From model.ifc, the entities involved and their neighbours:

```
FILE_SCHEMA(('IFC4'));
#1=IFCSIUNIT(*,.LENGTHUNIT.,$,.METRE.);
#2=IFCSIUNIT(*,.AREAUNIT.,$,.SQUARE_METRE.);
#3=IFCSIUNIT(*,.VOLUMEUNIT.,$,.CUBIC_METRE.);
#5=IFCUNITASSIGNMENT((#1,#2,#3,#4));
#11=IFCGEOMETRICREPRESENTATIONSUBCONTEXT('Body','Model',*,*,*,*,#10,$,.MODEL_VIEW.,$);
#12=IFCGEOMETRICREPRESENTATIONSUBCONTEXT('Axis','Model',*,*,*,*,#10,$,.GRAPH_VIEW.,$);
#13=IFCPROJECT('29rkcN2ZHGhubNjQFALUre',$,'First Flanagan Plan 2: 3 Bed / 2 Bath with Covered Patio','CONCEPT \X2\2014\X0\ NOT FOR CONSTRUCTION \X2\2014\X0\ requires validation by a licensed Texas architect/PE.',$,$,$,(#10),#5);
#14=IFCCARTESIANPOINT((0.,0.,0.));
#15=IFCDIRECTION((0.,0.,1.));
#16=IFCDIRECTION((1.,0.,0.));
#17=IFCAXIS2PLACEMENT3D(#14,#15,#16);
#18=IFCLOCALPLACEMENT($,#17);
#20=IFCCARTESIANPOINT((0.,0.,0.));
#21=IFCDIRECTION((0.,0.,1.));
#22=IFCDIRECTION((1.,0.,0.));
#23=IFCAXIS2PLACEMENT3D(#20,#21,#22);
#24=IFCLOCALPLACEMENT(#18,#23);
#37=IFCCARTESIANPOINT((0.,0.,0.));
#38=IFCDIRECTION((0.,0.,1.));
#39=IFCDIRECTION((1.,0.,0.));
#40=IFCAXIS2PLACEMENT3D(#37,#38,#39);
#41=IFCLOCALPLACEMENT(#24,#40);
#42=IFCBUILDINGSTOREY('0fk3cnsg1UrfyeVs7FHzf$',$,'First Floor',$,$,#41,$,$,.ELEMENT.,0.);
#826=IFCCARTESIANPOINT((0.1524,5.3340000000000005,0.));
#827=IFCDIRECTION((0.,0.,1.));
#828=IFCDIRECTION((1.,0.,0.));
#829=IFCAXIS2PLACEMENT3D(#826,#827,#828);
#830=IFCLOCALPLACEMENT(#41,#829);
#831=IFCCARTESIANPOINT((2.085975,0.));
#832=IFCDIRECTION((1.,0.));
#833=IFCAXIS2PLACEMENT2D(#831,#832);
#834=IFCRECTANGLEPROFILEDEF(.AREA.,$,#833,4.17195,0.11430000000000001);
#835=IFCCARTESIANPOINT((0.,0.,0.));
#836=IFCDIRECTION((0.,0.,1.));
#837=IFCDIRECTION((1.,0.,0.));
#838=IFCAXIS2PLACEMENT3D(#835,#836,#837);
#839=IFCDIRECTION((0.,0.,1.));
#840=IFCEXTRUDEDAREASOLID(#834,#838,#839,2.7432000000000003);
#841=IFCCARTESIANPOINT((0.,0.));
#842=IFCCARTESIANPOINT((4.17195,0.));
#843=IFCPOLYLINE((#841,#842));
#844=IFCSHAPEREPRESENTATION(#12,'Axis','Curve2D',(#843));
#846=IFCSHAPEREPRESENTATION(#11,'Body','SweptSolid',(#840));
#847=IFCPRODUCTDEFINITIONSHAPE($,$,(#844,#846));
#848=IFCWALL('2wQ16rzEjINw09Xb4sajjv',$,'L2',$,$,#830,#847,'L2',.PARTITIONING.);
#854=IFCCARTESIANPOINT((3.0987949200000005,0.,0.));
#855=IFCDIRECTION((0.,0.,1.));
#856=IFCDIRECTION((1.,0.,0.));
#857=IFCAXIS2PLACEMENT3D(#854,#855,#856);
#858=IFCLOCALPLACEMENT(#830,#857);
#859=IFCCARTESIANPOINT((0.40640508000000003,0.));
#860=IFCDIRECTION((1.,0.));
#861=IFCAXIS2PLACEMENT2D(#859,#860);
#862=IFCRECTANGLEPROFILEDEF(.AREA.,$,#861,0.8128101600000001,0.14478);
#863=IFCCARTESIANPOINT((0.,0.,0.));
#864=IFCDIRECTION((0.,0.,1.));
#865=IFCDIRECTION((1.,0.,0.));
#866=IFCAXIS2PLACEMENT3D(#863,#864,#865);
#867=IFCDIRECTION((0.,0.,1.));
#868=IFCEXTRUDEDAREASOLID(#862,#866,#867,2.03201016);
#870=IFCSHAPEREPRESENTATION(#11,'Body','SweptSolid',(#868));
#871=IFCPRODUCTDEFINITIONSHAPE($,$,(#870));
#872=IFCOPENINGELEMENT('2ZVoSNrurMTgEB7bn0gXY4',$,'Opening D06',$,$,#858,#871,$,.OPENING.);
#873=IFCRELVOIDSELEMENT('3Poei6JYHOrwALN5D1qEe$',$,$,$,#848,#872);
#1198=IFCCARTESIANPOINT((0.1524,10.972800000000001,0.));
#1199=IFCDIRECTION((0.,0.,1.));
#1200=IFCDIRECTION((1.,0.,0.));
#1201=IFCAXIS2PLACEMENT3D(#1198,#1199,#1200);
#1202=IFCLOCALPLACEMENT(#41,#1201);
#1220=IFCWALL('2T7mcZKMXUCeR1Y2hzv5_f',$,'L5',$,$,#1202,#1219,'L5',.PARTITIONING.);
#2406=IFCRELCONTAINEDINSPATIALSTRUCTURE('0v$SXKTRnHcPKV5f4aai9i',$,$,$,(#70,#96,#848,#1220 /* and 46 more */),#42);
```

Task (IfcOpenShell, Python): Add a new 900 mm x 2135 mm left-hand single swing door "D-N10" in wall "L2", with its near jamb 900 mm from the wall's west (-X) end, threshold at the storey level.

```python
import numpy as np
import ifcopenshell
import ifcopenshell.api.feature
import ifcopenshell.api.geometry
import ifcopenshell.api.root
import ifcopenshell.api.spatial
import ifcopenshell.geom
import ifcopenshell.util.element
import ifcopenshell.util.placement
import ifcopenshell.util.representation
import ifcopenshell.util.shape
import ifcopenshell.util.unit

model = ifcopenshell.open("model.ifc")
unit_scale = ifcopenshell.util.unit.calculate_unit_scale(model)
settings = ifcopenshell.geom.settings()


def volume(element):
    """Net volume in cubic metres, openings subtracted."""
    shape = ifcopenshell.geom.create_shape(settings, element)
    return ifcopenshell.util.shape.get_volume(shape.geometry)


wall = model.by_id(848)
storey = ifcopenshell.util.element.get_container(wall, ifc_class="IfcBuildingStorey")
context = ifcopenshell.util.representation.get_context(model, "Model", "Body", "MODEL_VIEW")
before = volume(wall)

width, height, from_end, sill = 0.9, 2.135, 0.9, 0.0  # metres

# The wall runs along its own X axis, and the end named is its -X end.
wall_shape = ifcopenshell.geom.create_shape(settings, wall)
x, y, z = ifcopenshell.util.shape.get_vertices(wall_shape.geometry).T
start = x.min() + from_end
face, thickness = float(y.min()), float(y.max() - y.min())
wall_matrix = ifcopenshell.util.placement.get_local_placement(wall.ObjectPlacement)
level = ifcopenshell.util.placement.get_local_placement(storey.ObjectPlacement)[2, 3]


def in_wall(x, y):
    """Placement at x, y metres in the wall's axes, at sill height."""
    matrix = wall_matrix.copy()
    matrix[:, 3] = wall_matrix @ np.array([x / unit_scale, y / unit_scale, 0.0, 1.0])
    matrix[2, 3] = level + sill / unit_scale
    return matrix


# Opening: a box that overshoots both wall faces by 50 mm.
opening = ifcopenshell.api.root.create_entity(model, ifc_class="IfcOpeningElement", predefined_type="OPENING")
box = ifcopenshell.api.geometry.add_wall_representation(
    model, context=context, length=width, height=height, thickness=thickness + 0.1
)
ifcopenshell.api.geometry.assign_representation(model, product=opening, representation=box)
ifcopenshell.api.geometry.edit_object_placement(model, product=opening, matrix=in_wall(start, face - 0.05), is_si=False)
ifcopenshell.api.feature.add_feature(model, feature=opening, element=wall)

door = ifcopenshell.api.root.create_entity(model, ifc_class="IfcDoor", name="D-N10", predefined_type="DOOR")
door.OverallWidth, door.OverallHeight = width / unit_scale, height / unit_scale
door.OperationType = "SINGLE_SWING_LEFT"
body = ifcopenshell.api.geometry.add_door_representation(
    model,
    context=context,
    overall_width=door.OverallWidth,
    overall_height=door.OverallHeight,
    operation_type="SINGLE_SWING_LEFT",
    lining_properties={"LiningDepth": thickness / unit_scale, "ThresholdDepth": thickness / unit_scale},
)
ifcopenshell.api.geometry.assign_representation(model, product=door, representation=body)
ifcopenshell.api.spatial.assign_container(model, products=[door], relating_structure=storey)
ifcopenshell.api.feature.add_filling(model, opening=opening, element=door)

# The lining spans the wall, so the door starts at the wall face.
ifcopenshell.api.geometry.edit_object_placement(model, product=door, matrix=in_wall(start, face), is_si=False)

after = volume(wall)

print(f"wall volume {before:.3f} -> {after:.3f} m3")

model.write("model_updated.ifc")
```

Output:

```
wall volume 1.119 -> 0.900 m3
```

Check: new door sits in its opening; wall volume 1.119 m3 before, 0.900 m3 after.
